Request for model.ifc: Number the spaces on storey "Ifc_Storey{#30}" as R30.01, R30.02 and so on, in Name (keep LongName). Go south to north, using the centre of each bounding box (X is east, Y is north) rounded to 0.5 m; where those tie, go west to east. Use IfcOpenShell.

First a look at what the model holds.

```python
import ifcopenshell
import ifcopenshell.util.element
import ifcopenshell.util.placement

model = ifcopenshell.open("model.ifc")
print(model.schema)
storey = next(s for s in model.by_type("IfcBuildingStorey") if s.Name == "Ifc_Storey{#30}")
spaces = [e for e in ifcopenshell.util.element.get_decomposition(storey) if e.is_a("IfcSpace")]
for e in sorted(spaces, key=lambda e: e.id()):
    origin = ifcopenshell.util.placement.get_local_placement(e.ObjectPlacement)[:3, 3]
    print(e.id(), e.Name, e.LongName, origin.round(2) + 0.0, sep=" | ")
```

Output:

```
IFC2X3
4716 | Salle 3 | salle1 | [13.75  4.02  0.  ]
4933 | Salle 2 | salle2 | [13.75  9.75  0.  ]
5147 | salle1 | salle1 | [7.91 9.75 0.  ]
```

```python
import ifcopenshell
import ifcopenshell.geom
import ifcopenshell.util.element
import ifcopenshell.util.shape

model = ifcopenshell.open("model.ifc")
settings = ifcopenshell.geom.settings()
settings.set("use-world-coords", True)


def centre(element):
    shape = ifcopenshell.geom.create_shape(settings, element)
    return ifcopenshell.util.shape.get_bbox_centroid(shape.geometry)


storey = next(s for s in model.by_type("IfcBuildingStorey") if s.Name == "Ifc_Storey{#30}")
spaces = [e for e in ifcopenshell.util.element.get_decomposition(storey) if e.is_a("IfcSpace")]

# Insertion points can sit at a corner or the storey origin, so sort by the geometry (in metres).
centres = {e: centre(e) for e in spaces}
spaces.sort(key=lambda e: (round(centres[e][1] / 0.5), centres[e][0]))

for i, e in enumerate(spaces, start=1):
    number = f"R30.{i:02d}"
    e.Name = number
    print(e.id(), number)

model.write("model_rev.ifc")
```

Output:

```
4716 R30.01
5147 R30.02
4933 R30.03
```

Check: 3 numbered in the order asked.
